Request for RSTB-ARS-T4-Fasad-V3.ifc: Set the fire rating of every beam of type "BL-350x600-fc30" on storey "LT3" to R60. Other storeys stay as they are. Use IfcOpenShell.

First a look at what the model holds.

```python
import ifcopenshell
import ifcopenshell.util.element

model = ifcopenshell.open("RSTB-ARS-T4-Fasad-V3.ifc")
print(model.schema)
storey = next(s for s in model.by_type("IfcBuildingStorey") if s.Name == "LT3")
beams = [e for e in ifcopenshell.util.element.get_decomposition(storey) if e.is_a("IfcBeam")]
seen = {}
for e in beams:
    element_type = ifcopenshell.util.element.get_type(e)
    key = (element_type.Name if element_type != e and element_type else None, ifcopenshell.util.element.get_pset(e, "Pset_BeamCommon", "FireRating"))
    seen[key] = seen.get(key, 0) + 1
for (name, value), count in sorted(seen.items(), key=str):
    print(count, "x", name, "|", value)
```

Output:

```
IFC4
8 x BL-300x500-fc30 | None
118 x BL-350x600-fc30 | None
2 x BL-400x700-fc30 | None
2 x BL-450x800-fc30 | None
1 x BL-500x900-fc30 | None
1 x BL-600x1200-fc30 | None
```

```python
import ifcopenshell
import ifcopenshell.api.pset
import ifcopenshell.util.element

model = ifcopenshell.open("RSTB-ARS-T4-Fasad-V3.ifc")

storey = next(s for s in model.by_type("IfcBuildingStorey") if s.Name == "LT3")
beams = [e for e in ifcopenshell.util.element.get_decomposition(storey) if e.is_a("IfcBeam")]

count = 0
for e in beams:
    element_type = ifcopenshell.util.element.get_type(e)
    if element_type in (None, e) or element_type.Name != "BL-350x600-fc30":
        continue
    # add_pset returns the element's existing set when there is one.
    pset = ifcopenshell.api.pset.add_pset(model, product=e, name="Pset_BeamCommon")
    ifcopenshell.api.pset.edit_pset(model, pset=pset, properties={"FireRating": "R60"})
    count += 1

print(count, "beams updated")

model.write("RSTB-ARS-T4-Fasad-V3-out.ifc")
```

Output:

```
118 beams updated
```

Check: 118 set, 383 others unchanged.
